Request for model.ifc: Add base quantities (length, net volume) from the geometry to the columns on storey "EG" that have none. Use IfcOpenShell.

First a look at what the model holds.

```python
import ifcopenshell
import ifcopenshell.util.element
import ifcopenshell.util.unit

model = ifcopenshell.open("model.ifc")
print(model.schema)
for unit_type in ("LENGTHUNIT", "AREAUNIT", "VOLUMEUNIT"):
    print(unit_type, ifcopenshell.util.unit.calculate_unit_scale(model, unit_type))
storey = next(s for s in model.by_type("IfcBuildingStorey") if s.Name == "EG")
columns = [e for e in ifcopenshell.util.element.get_decomposition(storey) if e.is_a("IfcColumn")]
for e in sorted(columns, key=lambda e: e.id()):
    print(e.id(), e.is_a(), e.Name, list(ifcopenshell.util.element.get_psets(e, qtos_only=True)), sep=" | ")
```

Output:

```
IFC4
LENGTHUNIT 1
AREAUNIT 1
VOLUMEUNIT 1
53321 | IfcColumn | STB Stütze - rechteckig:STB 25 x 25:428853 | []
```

```python
import ifcopenshell
import ifcopenshell.api.pset
import ifcopenshell.geom
import ifcopenshell.util.element
import ifcopenshell.util.shape
import ifcopenshell.util.unit

model = ifcopenshell.open("model.ifc")
unit_scale = ifcopenshell.util.unit.calculate_unit_scale(model)
volume_scale = ifcopenshell.util.unit.calculate_unit_scale(model, "VOLUMEUNIT")
settings = ifcopenshell.geom.settings()

storey = next(s for s in model.by_type("IfcBuildingStorey") if s.Name == "EG")
columns = [e for e in ifcopenshell.util.element.get_decomposition(storey) if e.is_a("IfcColumn")]

for e in sorted(columns, key=lambda e: e.id()):
    if ifcopenshell.util.element.get_psets(e, qtos_only=True, should_inherit=False):
        continue
    # Geometry comes back in metres, in the element's own axes.
    shape = ifcopenshell.geom.create_shape(settings, e)
    values = {
        "Length": ifcopenshell.util.shape.get_z(shape.geometry) / unit_scale,
        "NetVolume": ifcopenshell.util.shape.get_volume(shape.geometry) / volume_scale,
    }
    qto = ifcopenshell.api.pset.add_qto(model, product=e, name="Qto_ColumnBaseQuantities")
    ifcopenshell.api.pset.edit_qto(model, qto=qto, properties=values)
    print(e.id(), {k: round(v, 3) for k, v in values.items()})

model.write("model-out.ifc")
```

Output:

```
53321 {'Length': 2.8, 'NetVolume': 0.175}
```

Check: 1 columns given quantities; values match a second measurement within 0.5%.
